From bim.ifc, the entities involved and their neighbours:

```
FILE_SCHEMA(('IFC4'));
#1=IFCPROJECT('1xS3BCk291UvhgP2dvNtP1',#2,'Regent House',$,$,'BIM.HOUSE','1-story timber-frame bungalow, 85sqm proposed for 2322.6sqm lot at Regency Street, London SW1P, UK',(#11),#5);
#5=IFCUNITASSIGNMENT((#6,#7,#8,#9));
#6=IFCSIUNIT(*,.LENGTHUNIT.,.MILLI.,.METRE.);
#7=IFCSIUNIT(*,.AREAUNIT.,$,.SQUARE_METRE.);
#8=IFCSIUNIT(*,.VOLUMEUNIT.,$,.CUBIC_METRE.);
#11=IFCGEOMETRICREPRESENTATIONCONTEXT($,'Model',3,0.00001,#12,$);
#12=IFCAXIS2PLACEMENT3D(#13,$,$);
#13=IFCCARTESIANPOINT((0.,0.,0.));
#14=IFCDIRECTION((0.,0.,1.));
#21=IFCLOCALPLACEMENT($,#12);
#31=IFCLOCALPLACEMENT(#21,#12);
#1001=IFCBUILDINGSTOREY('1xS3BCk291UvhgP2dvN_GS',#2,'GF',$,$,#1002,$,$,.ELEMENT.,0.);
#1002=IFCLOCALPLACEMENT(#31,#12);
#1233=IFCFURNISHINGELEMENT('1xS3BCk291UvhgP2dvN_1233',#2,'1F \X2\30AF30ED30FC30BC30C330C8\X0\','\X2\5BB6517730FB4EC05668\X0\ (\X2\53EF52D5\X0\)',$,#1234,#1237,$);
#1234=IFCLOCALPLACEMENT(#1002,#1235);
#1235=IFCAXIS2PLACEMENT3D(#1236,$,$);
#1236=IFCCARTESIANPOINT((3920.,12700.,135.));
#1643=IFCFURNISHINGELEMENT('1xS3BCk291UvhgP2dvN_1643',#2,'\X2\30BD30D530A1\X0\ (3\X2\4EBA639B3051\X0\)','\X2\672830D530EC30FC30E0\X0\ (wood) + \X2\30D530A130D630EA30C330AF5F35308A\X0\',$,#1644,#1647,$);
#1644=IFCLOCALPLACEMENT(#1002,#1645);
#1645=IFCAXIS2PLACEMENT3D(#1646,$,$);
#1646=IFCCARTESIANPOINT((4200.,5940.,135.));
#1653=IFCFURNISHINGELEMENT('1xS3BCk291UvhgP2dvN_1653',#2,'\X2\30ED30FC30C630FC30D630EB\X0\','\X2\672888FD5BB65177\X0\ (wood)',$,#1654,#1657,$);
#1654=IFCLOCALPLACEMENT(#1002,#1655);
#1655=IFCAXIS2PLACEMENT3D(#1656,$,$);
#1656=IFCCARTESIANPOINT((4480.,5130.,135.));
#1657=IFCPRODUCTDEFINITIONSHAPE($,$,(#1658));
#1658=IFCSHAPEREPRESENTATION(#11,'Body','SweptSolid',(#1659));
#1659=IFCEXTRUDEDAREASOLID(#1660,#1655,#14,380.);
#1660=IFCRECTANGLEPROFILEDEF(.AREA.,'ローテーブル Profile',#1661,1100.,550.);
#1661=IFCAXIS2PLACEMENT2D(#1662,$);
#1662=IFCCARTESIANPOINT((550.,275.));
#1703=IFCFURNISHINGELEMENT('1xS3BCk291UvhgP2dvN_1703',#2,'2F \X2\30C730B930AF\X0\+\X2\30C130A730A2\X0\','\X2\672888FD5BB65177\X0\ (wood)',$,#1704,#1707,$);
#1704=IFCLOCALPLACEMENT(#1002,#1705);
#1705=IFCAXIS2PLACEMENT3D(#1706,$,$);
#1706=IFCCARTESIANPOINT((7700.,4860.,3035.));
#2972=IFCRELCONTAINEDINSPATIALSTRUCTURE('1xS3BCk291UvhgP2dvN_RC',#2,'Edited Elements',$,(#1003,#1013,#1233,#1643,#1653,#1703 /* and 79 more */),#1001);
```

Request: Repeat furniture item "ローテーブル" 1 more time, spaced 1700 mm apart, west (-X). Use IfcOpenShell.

```python
import numpy as np
import ifcopenshell
import ifcopenshell.api.geometry
import ifcopenshell.api.root
import ifcopenshell.util.element
import ifcopenshell.util.placement
import ifcopenshell.util.unit

model = ifcopenshell.open("bim.ifc")
unit_scale = ifcopenshell.util.unit.calculate_unit_scale(model)


def reuse_history(source, copy):
    """copy_class also copies each property set's owner history, people and application; keep the originals."""
    for rel in copy.IsDefinedBy:
        if rel.is_a("IfcRelDefinesByProperties") and (history := rel.RelatingPropertyDefinition.OwnerHistory):
            rel.RelatingPropertyDefinition.OwnerHistory = source.OwnerHistory
            ifcopenshell.util.element.remove_deep2(model, history)


source = model.by_guid("1xS3BCk291UvhgP2dvN_1653")
base = ifcopenshell.util.placement.get_local_placement(source.ObjectPlacement)
step = np.array([-1.0, 0.0, 0.0]) * 1.7 / unit_scale

for i in range(1, 2):
    copy = ifcopenshell.api.root.copy_class(model, product=source)
    copy.Representation = ifcopenshell.util.element.copy_deep(
        model, source.Representation, exclude=["IfcGeometricRepresentationContext", "IfcRepresentationMap"]
    )
    reuse_history(source, copy)
    matrix = base.copy()
    matrix[:3, 3] += i * step
    print("added at", matrix[:3, 3].round(3) + 0.0)
    ifcopenshell.api.geometry.edit_object_placement(model, product=copy, matrix=matrix, is_si=False)

model.write("bim_edited.ifc")
```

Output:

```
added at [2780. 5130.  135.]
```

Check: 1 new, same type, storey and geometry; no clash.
